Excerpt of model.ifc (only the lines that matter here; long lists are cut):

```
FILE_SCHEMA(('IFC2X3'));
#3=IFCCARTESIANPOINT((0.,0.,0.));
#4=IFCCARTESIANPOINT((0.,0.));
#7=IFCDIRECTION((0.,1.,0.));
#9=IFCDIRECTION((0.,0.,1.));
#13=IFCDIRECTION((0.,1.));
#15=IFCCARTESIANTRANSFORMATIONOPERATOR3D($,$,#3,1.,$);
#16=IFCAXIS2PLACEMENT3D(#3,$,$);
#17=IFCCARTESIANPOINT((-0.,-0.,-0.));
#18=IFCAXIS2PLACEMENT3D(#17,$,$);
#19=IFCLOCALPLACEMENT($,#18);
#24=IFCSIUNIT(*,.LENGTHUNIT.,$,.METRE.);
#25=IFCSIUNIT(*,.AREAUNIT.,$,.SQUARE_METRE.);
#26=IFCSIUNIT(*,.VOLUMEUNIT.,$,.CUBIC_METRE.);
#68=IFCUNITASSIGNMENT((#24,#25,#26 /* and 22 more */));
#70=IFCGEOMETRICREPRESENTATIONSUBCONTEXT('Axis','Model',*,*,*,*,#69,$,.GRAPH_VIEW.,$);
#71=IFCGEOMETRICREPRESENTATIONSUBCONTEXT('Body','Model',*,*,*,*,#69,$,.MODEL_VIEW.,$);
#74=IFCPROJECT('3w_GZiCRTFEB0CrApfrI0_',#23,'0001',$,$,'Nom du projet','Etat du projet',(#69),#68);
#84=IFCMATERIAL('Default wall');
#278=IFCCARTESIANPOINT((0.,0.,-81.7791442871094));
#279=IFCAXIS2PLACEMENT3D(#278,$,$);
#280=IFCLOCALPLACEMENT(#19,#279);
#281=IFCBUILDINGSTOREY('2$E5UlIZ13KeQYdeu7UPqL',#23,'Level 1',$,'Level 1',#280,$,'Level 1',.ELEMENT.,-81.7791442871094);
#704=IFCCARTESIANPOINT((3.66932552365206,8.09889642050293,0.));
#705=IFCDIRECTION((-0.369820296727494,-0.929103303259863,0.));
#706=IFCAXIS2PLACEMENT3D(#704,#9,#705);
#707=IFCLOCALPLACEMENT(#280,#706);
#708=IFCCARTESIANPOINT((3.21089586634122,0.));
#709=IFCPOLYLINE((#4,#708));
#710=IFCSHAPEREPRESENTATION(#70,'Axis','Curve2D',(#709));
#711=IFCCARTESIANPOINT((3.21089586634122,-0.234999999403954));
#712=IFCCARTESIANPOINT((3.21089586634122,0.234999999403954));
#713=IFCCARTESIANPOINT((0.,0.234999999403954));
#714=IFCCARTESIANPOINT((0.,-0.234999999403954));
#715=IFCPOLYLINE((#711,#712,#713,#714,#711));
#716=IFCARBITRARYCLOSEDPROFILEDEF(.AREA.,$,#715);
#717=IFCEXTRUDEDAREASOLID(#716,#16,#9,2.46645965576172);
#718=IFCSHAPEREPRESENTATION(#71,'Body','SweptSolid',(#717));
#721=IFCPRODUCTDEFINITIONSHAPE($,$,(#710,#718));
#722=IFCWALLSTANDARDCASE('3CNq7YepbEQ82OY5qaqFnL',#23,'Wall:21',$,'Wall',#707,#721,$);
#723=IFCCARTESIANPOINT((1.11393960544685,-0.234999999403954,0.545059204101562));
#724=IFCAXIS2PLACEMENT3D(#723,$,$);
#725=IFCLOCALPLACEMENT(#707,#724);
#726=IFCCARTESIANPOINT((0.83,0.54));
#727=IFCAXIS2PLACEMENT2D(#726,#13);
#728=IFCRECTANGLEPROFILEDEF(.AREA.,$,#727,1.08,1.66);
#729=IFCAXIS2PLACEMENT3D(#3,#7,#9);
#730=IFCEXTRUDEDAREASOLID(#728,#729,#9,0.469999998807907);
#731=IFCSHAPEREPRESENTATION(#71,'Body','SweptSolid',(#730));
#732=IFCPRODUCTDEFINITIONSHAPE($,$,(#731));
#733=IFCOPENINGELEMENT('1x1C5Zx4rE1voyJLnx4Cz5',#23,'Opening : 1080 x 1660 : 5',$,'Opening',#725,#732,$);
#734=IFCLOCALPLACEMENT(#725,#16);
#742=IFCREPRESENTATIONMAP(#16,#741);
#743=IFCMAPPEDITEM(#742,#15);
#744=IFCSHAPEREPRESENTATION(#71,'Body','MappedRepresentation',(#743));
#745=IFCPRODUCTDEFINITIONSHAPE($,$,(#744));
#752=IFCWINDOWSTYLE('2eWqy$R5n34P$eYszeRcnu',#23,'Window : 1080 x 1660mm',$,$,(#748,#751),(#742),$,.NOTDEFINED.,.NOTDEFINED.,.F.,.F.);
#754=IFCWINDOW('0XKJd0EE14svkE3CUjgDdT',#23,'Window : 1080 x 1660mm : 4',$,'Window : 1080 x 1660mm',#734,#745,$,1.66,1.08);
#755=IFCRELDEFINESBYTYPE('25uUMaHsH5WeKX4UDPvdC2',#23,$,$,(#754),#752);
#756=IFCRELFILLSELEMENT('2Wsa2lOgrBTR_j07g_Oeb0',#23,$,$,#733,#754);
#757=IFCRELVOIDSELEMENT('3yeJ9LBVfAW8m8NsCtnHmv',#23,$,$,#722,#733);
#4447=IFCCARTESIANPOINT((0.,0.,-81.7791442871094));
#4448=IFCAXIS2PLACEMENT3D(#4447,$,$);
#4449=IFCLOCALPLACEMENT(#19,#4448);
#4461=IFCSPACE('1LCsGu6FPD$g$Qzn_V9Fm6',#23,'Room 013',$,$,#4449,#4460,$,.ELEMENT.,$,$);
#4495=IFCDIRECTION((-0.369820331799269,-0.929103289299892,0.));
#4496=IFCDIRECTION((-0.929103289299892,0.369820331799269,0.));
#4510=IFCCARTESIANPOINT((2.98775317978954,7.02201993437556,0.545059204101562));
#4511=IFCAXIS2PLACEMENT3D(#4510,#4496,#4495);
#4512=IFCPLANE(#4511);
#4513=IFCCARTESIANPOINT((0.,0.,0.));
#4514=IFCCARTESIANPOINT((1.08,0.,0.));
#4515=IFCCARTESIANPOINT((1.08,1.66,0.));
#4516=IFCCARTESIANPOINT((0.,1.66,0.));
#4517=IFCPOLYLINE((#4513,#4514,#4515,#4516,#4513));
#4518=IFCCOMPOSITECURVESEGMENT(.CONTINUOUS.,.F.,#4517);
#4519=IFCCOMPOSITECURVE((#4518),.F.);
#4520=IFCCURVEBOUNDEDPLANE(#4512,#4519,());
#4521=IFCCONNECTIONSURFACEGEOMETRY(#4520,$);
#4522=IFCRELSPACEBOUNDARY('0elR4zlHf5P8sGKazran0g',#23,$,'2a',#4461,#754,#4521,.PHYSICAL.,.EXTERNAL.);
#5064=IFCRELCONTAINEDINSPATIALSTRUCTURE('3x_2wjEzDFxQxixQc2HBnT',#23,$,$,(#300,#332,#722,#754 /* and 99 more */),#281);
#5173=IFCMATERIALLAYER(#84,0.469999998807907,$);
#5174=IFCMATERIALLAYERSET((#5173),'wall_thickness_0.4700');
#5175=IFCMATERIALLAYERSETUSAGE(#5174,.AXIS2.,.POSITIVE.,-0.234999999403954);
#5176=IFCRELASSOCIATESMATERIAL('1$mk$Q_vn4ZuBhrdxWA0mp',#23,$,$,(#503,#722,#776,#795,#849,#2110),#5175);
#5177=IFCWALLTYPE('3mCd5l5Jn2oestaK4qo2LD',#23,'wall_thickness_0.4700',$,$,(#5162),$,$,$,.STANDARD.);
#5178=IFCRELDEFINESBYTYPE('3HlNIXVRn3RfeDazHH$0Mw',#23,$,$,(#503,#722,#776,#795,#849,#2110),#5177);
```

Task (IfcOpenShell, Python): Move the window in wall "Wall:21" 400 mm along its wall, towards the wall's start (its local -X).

```python
import numpy as np
import ifcopenshell
import ifcopenshell.api.geometry
import ifcopenshell.util.placement
import ifcopenshell.util.unit

model = ifcopenshell.open("model.ifc")
unit_scale = ifcopenshell.util.unit.calculate_unit_scale(model)

window = model.by_id(754)
opening = window.FillsVoids[0].RelatingOpeningElement
wall = opening.VoidsElements[0].RelatingBuildingElement

wall_matrix = ifcopenshell.util.placement.get_local_placement(wall.ObjectPlacement)
shift = wall_matrix[:3, 0] * -0.4 / unit_scale
before = ifcopenshell.util.placement.get_local_placement(window.ObjectPlacement)[:3, 3].copy()

# The window is placed relative to its opening, so it follows when the opening moves.
matrix = ifcopenshell.util.placement.get_local_placement(opening.ObjectPlacement)
matrix[:3, 3] += shift
ifcopenshell.api.geometry.edit_object_placement(
    model, product=opening, matrix=matrix, is_si=False, should_transform_children=True
)

# Space boundary surfaces are stored in each space's coordinates; move them too.
for rel in window.ProvidesBoundaries:
    if not rel.ConnectionGeometry:
        continue
    surface = rel.ConnectionGeometry.SurfaceOnRelatingElement.BasisSurface
    space_matrix = ifcopenshell.util.placement.get_local_placement(rel.RelatingSpace.ObjectPlacement)
    point = np.array(surface.Position.Location.Coordinates) + space_matrix[:3, :3].T @ shift
    surface.Position = model.createIfcAxis2Placement3D(
        model.createIfcCartesianPoint(point.tolist()), surface.Position.Axis, surface.Position.RefDirection
    )

after = ifcopenshell.util.placement.get_local_placement(window.ObjectPlacement)[:3, 3]
print("window moved by", (after - before).round(3) + 0.0)

model.write("model_edited.ifc")
```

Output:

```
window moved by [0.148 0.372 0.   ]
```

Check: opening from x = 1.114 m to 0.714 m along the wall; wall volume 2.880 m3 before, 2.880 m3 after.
